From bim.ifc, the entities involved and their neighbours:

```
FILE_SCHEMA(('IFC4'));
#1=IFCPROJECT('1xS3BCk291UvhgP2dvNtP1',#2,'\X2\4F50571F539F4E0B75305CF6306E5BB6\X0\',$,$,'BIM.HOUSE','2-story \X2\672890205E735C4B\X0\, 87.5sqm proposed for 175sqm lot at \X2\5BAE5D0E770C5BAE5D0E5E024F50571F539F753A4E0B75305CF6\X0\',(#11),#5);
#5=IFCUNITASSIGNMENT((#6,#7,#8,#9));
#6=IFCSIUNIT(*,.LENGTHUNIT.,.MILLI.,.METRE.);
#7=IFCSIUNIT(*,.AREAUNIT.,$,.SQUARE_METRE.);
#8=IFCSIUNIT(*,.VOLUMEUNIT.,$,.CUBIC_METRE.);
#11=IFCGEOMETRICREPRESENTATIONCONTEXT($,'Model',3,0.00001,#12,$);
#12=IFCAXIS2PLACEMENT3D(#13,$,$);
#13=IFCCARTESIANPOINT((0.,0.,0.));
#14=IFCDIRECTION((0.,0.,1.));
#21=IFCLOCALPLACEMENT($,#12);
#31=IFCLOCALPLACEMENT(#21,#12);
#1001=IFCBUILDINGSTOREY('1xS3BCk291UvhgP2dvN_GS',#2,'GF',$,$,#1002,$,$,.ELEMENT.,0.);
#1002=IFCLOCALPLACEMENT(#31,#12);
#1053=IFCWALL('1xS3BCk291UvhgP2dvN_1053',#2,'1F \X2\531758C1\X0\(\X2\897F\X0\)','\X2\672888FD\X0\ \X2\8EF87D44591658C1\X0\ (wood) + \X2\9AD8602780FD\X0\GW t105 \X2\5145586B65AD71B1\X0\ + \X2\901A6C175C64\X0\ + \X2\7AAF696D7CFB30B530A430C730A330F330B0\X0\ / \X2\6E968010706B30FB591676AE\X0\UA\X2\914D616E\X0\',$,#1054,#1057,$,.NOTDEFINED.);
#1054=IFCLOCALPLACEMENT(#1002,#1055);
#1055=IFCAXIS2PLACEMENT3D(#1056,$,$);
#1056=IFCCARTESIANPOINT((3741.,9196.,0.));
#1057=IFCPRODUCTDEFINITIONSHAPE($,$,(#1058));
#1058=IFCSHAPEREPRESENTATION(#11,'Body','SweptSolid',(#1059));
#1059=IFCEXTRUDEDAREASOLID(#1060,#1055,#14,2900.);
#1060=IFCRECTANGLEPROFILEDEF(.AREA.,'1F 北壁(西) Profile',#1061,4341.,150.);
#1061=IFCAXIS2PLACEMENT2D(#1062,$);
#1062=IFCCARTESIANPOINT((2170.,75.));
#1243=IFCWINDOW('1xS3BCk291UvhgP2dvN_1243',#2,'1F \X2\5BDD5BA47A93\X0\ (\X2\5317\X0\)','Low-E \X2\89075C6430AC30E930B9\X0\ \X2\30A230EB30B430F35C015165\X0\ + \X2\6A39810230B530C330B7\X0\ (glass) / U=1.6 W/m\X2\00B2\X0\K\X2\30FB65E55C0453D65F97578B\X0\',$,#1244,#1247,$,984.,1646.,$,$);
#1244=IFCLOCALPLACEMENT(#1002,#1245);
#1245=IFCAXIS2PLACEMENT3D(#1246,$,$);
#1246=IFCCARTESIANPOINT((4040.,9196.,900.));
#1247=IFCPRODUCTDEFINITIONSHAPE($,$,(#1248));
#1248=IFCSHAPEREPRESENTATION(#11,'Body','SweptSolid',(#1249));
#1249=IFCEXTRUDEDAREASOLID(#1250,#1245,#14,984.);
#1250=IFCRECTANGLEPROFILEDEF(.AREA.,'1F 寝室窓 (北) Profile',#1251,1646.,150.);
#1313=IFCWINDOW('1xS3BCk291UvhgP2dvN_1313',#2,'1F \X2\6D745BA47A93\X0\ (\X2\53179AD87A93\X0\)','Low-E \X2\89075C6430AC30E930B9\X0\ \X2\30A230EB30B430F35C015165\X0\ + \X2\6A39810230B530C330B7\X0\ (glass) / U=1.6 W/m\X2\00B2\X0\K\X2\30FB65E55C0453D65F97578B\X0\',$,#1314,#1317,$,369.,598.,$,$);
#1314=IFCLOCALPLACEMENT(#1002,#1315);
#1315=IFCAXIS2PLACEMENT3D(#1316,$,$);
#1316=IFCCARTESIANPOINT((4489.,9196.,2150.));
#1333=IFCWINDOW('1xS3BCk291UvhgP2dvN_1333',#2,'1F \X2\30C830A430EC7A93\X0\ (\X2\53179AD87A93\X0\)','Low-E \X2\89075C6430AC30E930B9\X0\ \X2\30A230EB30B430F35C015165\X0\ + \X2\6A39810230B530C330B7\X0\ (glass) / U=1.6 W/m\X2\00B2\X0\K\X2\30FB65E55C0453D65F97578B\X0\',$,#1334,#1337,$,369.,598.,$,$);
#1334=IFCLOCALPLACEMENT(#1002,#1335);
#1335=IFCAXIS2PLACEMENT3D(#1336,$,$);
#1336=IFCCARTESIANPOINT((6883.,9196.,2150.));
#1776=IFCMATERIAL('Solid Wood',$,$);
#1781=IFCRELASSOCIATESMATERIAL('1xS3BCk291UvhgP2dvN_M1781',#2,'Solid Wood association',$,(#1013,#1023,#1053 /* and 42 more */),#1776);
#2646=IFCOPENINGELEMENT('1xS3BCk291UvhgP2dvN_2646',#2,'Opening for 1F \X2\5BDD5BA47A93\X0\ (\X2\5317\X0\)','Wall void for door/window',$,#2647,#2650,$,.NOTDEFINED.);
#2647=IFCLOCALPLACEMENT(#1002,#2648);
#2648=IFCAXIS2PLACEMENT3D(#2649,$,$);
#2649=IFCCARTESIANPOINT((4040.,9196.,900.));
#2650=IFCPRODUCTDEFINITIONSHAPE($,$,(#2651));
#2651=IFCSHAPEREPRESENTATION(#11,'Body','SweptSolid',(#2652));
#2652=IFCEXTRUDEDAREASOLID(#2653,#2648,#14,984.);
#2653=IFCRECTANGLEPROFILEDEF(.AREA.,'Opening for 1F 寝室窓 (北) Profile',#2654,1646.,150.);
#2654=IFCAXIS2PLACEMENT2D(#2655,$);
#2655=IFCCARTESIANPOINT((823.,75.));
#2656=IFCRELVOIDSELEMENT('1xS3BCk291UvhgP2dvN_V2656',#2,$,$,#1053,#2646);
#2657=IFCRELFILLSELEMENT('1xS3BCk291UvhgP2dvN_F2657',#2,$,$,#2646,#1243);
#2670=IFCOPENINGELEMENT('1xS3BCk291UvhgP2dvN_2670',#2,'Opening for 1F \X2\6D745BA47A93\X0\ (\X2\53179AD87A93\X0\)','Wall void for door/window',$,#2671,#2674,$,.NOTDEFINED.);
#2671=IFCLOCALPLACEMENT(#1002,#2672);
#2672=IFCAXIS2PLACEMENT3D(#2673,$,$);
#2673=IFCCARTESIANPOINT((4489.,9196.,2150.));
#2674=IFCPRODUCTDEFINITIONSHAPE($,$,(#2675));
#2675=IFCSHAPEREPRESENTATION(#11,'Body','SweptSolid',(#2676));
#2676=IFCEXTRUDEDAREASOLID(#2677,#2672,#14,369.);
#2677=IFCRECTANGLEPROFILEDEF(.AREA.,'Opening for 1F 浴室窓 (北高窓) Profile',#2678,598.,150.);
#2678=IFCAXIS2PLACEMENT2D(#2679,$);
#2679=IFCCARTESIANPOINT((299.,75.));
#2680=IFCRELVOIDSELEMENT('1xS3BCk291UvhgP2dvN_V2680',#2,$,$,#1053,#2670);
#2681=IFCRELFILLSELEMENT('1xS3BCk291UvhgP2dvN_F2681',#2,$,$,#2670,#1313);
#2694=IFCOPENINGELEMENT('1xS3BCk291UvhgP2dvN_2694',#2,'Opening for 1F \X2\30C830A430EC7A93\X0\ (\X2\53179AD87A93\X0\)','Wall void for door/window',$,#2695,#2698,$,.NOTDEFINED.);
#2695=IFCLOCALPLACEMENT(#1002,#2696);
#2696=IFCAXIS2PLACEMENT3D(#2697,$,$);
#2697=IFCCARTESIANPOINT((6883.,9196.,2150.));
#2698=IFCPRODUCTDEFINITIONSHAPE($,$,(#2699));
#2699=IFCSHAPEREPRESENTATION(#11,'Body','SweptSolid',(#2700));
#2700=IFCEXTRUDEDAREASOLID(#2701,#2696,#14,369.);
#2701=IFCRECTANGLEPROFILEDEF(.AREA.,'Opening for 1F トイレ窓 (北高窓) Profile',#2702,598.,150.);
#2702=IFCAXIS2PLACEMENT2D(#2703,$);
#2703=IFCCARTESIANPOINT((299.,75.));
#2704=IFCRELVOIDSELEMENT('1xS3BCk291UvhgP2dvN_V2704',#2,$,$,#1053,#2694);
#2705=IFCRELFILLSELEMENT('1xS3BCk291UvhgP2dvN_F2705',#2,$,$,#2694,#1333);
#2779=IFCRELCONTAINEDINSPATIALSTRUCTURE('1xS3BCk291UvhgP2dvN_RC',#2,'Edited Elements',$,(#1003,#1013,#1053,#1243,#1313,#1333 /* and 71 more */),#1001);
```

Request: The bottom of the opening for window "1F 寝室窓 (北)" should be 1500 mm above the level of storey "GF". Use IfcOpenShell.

```python
import numpy as np
import ifcopenshell
import ifcopenshell.api.geometry
import ifcopenshell.geom
import ifcopenshell.util.element
import ifcopenshell.util.placement
import ifcopenshell.util.shape
import ifcopenshell.util.unit

model = ifcopenshell.open("bim.ifc")
unit_scale = ifcopenshell.util.unit.calculate_unit_scale(model)

window = model.by_guid("1xS3BCk291UvhgP2dvN_1243")
opening = window.FillsVoids[0].RelatingOpeningElement
storey = ifcopenshell.util.element.get_container(window, ifc_class="IfcBuildingStorey")
level = ifcopenshell.util.placement.get_local_placement(storey.ObjectPlacement)[2, 3]

# The opening's origin need not be at the sill, so measure its lowest point.
shape = ifcopenshell.geom.create_shape(ifcopenshell.geom.settings(), opening)
bottom = ifcopenshell.util.shape.get_shape_bottom_elevation(shape, shape.geometry) / unit_scale
dz = level + 1.5 / unit_scale - bottom

shift = np.array([0.0, 0.0, dz])
# The window is not placed relative to its opening, so move both.
for product in (opening, window):
    matrix = ifcopenshell.util.placement.get_local_placement(product.ObjectPlacement)
    matrix[:3, 3] += shift
    ifcopenshell.api.geometry.edit_object_placement(model, product=product, matrix=matrix, is_si=False)

print(f"moved by {dz * unit_scale:+.3f} m")

model.write("bim_updated.ifc")
```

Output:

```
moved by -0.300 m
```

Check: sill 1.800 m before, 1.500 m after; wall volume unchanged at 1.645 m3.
